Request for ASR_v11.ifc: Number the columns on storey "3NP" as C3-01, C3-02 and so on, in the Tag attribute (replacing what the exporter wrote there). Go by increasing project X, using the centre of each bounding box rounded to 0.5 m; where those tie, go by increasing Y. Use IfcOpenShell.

First a look at what the model holds.

```python
import ifcopenshell
import ifcopenshell.util.element
import ifcopenshell.util.placement

model = ifcopenshell.open("ASR_v11.ifc")
print(model.schema)
storey = next(s for s in model.by_type("IfcBuildingStorey") if s.Name == "3NP")
columns = [e for e in ifcopenshell.util.element.get_decomposition(storey) if e.is_a("IfcColumn")]
for e in sorted(columns, key=lambda e: e.id()):
    origin = ifcopenshell.util.placement.get_local_placement(e.ObjectPlacement)[:3, 3]
    print(e.id(), e.Tag, e.Name, origin.round(2) + 0.0, sep=" | ")
```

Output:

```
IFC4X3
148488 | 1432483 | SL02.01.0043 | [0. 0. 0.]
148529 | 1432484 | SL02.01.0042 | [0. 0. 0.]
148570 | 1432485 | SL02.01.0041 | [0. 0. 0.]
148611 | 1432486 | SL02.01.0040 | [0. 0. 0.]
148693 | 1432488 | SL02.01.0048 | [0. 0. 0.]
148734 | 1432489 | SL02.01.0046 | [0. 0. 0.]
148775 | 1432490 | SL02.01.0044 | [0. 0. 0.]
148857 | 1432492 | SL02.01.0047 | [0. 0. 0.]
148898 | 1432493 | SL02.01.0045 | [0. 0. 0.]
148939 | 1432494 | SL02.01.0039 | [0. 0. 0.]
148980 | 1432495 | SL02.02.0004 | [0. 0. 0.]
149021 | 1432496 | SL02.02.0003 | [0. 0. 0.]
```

```python
import ifcopenshell
import ifcopenshell.geom
import ifcopenshell.util.element
import ifcopenshell.util.shape

model = ifcopenshell.open("ASR_v11.ifc")
settings = ifcopenshell.geom.settings()
settings.set("use-world-coords", True)


def centre(element):
    shape = ifcopenshell.geom.create_shape(settings, element)
    return ifcopenshell.util.shape.get_bbox_centroid(shape.geometry)


storey = next(s for s in model.by_type("IfcBuildingStorey") if s.Name == "3NP")
columns = [e for e in ifcopenshell.util.element.get_decomposition(storey) if e.is_a("IfcColumn")]

# Insertion points can sit at a corner or the storey origin, so sort by the geometry (in metres).
centres = {e: centre(e) for e in columns}
columns.sort(key=lambda e: (round(centres[e][0] / 0.5), centres[e][1]))

for i, e in enumerate(columns, start=1):
    number = f"C3-{i:02d}"
    e.Tag = number
    print(e.id(), number)

model.write("ASR_v11_v2.ifc")
```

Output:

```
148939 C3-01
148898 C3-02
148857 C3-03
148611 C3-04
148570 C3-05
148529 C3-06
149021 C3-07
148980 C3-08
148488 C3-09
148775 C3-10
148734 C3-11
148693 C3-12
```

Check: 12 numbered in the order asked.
